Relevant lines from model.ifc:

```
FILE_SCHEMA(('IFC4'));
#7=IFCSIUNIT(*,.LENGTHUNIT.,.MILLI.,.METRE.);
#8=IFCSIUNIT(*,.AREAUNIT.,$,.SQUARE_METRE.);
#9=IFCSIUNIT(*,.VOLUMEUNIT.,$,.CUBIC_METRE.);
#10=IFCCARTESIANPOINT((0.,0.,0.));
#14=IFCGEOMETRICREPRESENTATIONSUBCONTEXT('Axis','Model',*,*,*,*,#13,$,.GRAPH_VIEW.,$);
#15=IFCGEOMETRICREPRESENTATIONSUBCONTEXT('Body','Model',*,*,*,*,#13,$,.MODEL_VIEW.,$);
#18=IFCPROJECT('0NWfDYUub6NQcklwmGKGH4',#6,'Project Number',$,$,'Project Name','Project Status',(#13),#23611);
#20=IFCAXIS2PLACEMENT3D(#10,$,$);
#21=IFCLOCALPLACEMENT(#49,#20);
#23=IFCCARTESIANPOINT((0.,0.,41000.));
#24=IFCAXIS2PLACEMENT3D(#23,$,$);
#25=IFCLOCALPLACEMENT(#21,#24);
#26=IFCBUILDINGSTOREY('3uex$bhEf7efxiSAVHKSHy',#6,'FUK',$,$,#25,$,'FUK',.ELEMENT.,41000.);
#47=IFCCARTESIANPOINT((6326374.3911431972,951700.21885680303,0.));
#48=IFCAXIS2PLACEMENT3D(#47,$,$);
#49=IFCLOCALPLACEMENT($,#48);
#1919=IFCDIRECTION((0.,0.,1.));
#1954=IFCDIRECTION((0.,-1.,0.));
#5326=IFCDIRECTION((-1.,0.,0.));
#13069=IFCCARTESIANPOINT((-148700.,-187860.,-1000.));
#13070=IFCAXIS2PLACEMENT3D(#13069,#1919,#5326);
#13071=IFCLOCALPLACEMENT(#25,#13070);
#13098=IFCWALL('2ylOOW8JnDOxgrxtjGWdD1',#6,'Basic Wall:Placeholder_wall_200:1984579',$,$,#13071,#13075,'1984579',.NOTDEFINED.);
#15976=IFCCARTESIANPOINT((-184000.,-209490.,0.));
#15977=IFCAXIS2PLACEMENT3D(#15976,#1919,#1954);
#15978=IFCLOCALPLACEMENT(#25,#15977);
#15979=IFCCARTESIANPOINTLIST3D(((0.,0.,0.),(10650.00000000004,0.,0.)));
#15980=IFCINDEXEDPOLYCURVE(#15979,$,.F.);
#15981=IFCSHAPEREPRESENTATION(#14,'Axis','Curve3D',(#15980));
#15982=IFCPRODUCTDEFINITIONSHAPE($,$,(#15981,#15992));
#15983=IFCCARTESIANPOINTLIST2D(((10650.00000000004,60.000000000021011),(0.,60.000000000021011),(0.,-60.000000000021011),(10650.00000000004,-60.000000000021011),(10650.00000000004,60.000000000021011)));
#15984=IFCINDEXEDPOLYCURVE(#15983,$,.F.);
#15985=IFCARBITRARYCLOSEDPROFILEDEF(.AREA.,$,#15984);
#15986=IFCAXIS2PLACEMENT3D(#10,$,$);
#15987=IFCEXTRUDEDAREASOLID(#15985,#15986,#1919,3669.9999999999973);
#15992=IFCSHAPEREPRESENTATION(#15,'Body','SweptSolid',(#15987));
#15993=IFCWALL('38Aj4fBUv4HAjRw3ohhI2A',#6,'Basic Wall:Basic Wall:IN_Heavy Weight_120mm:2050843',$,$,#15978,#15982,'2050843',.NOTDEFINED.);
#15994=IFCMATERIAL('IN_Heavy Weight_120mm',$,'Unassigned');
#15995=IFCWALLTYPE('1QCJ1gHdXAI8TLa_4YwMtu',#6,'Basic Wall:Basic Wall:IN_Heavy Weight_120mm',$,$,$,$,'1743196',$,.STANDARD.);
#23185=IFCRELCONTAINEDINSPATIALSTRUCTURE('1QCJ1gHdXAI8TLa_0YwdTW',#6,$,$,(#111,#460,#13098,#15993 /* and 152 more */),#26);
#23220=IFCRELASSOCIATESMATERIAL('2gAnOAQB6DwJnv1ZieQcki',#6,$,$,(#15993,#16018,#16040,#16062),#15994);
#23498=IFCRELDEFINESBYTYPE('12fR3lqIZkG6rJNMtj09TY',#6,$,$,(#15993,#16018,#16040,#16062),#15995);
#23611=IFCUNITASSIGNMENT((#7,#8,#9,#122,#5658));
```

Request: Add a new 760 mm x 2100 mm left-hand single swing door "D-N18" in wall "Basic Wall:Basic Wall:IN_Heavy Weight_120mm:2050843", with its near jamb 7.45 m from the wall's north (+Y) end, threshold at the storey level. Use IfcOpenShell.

```python
import numpy as np
import ifcopenshell
import ifcopenshell.api.feature
import ifcopenshell.api.geometry
import ifcopenshell.api.root
import ifcopenshell.api.spatial
import ifcopenshell.geom
import ifcopenshell.util.element
import ifcopenshell.util.placement
import ifcopenshell.util.representation
import ifcopenshell.util.shape
import ifcopenshell.util.unit

model = ifcopenshell.open("model.ifc")
unit_scale = ifcopenshell.util.unit.calculate_unit_scale(model)
settings = ifcopenshell.geom.settings()


def volume(element):
    """Net volume in cubic metres, openings subtracted."""
    shape = ifcopenshell.geom.create_shape(settings, element)
    return ifcopenshell.util.shape.get_volume(shape.geometry)


wall = model.by_guid("38Aj4fBUv4HAjRw3ohhI2A")
storey = ifcopenshell.util.element.get_container(wall, ifc_class="IfcBuildingStorey")
context = ifcopenshell.util.representation.get_context(model, "Model", "Body", "MODEL_VIEW")
before = volume(wall)

width, height, from_end, sill = 0.76, 2.1, 7.45, 0.0  # metres

# The wall runs along its own X axis, and the end named is its -X end.
wall_shape = ifcopenshell.geom.create_shape(settings, wall)
x, y, z = ifcopenshell.util.shape.get_vertices(wall_shape.geometry).T
start = x.min() + from_end
face, thickness = float(y.min()), float(y.max() - y.min())
wall_matrix = ifcopenshell.util.placement.get_local_placement(wall.ObjectPlacement)
level = ifcopenshell.util.placement.get_local_placement(storey.ObjectPlacement)[2, 3]


def in_wall(x, y):
    """Placement at x, y metres in the wall's axes, at sill height."""
    matrix = wall_matrix.copy()
    matrix[:, 3] = wall_matrix @ np.array([x / unit_scale, y / unit_scale, 0.0, 1.0])
    matrix[2, 3] = level + sill / unit_scale
    return matrix


# Opening: a box that overshoots both wall faces by 50 mm.
opening = ifcopenshell.api.root.create_entity(model, ifc_class="IfcOpeningElement", predefined_type="OPENING")
box = ifcopenshell.api.geometry.add_wall_representation(
    model, context=context, length=width, height=height, thickness=thickness + 0.1
)
ifcopenshell.api.geometry.assign_representation(model, product=opening, representation=box)
ifcopenshell.api.geometry.edit_object_placement(model, product=opening, matrix=in_wall(start, face - 0.05), is_si=False)
ifcopenshell.api.feature.add_feature(model, feature=opening, element=wall)

door = ifcopenshell.api.root.create_entity(model, ifc_class="IfcDoor", name="D-N18", predefined_type="DOOR")
door.OverallWidth, door.OverallHeight = width / unit_scale, height / unit_scale
door.OperationType = "SINGLE_SWING_LEFT"
body = ifcopenshell.api.geometry.add_door_representation(
    model,
    context=context,
    overall_width=door.OverallWidth,
    overall_height=door.OverallHeight,
    operation_type="SINGLE_SWING_LEFT",
    lining_properties={"LiningDepth": thickness / unit_scale, "ThresholdDepth": thickness / unit_scale},
)
ifcopenshell.api.geometry.assign_representation(model, product=door, representation=body)
ifcopenshell.api.spatial.assign_container(model, products=[door], relating_structure=storey)
ifcopenshell.api.feature.add_filling(model, opening=opening, element=door)

# The lining spans the wall, so the door starts at the wall face.
ifcopenshell.api.geometry.edit_object_placement(model, product=door, matrix=in_wall(start, face), is_si=False)

after = volume(wall)

print(f"wall volume {before:.3f} -> {after:.3f} m3")

model.write("model_edited.ifc")
```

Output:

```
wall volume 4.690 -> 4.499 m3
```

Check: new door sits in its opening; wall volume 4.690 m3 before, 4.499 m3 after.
